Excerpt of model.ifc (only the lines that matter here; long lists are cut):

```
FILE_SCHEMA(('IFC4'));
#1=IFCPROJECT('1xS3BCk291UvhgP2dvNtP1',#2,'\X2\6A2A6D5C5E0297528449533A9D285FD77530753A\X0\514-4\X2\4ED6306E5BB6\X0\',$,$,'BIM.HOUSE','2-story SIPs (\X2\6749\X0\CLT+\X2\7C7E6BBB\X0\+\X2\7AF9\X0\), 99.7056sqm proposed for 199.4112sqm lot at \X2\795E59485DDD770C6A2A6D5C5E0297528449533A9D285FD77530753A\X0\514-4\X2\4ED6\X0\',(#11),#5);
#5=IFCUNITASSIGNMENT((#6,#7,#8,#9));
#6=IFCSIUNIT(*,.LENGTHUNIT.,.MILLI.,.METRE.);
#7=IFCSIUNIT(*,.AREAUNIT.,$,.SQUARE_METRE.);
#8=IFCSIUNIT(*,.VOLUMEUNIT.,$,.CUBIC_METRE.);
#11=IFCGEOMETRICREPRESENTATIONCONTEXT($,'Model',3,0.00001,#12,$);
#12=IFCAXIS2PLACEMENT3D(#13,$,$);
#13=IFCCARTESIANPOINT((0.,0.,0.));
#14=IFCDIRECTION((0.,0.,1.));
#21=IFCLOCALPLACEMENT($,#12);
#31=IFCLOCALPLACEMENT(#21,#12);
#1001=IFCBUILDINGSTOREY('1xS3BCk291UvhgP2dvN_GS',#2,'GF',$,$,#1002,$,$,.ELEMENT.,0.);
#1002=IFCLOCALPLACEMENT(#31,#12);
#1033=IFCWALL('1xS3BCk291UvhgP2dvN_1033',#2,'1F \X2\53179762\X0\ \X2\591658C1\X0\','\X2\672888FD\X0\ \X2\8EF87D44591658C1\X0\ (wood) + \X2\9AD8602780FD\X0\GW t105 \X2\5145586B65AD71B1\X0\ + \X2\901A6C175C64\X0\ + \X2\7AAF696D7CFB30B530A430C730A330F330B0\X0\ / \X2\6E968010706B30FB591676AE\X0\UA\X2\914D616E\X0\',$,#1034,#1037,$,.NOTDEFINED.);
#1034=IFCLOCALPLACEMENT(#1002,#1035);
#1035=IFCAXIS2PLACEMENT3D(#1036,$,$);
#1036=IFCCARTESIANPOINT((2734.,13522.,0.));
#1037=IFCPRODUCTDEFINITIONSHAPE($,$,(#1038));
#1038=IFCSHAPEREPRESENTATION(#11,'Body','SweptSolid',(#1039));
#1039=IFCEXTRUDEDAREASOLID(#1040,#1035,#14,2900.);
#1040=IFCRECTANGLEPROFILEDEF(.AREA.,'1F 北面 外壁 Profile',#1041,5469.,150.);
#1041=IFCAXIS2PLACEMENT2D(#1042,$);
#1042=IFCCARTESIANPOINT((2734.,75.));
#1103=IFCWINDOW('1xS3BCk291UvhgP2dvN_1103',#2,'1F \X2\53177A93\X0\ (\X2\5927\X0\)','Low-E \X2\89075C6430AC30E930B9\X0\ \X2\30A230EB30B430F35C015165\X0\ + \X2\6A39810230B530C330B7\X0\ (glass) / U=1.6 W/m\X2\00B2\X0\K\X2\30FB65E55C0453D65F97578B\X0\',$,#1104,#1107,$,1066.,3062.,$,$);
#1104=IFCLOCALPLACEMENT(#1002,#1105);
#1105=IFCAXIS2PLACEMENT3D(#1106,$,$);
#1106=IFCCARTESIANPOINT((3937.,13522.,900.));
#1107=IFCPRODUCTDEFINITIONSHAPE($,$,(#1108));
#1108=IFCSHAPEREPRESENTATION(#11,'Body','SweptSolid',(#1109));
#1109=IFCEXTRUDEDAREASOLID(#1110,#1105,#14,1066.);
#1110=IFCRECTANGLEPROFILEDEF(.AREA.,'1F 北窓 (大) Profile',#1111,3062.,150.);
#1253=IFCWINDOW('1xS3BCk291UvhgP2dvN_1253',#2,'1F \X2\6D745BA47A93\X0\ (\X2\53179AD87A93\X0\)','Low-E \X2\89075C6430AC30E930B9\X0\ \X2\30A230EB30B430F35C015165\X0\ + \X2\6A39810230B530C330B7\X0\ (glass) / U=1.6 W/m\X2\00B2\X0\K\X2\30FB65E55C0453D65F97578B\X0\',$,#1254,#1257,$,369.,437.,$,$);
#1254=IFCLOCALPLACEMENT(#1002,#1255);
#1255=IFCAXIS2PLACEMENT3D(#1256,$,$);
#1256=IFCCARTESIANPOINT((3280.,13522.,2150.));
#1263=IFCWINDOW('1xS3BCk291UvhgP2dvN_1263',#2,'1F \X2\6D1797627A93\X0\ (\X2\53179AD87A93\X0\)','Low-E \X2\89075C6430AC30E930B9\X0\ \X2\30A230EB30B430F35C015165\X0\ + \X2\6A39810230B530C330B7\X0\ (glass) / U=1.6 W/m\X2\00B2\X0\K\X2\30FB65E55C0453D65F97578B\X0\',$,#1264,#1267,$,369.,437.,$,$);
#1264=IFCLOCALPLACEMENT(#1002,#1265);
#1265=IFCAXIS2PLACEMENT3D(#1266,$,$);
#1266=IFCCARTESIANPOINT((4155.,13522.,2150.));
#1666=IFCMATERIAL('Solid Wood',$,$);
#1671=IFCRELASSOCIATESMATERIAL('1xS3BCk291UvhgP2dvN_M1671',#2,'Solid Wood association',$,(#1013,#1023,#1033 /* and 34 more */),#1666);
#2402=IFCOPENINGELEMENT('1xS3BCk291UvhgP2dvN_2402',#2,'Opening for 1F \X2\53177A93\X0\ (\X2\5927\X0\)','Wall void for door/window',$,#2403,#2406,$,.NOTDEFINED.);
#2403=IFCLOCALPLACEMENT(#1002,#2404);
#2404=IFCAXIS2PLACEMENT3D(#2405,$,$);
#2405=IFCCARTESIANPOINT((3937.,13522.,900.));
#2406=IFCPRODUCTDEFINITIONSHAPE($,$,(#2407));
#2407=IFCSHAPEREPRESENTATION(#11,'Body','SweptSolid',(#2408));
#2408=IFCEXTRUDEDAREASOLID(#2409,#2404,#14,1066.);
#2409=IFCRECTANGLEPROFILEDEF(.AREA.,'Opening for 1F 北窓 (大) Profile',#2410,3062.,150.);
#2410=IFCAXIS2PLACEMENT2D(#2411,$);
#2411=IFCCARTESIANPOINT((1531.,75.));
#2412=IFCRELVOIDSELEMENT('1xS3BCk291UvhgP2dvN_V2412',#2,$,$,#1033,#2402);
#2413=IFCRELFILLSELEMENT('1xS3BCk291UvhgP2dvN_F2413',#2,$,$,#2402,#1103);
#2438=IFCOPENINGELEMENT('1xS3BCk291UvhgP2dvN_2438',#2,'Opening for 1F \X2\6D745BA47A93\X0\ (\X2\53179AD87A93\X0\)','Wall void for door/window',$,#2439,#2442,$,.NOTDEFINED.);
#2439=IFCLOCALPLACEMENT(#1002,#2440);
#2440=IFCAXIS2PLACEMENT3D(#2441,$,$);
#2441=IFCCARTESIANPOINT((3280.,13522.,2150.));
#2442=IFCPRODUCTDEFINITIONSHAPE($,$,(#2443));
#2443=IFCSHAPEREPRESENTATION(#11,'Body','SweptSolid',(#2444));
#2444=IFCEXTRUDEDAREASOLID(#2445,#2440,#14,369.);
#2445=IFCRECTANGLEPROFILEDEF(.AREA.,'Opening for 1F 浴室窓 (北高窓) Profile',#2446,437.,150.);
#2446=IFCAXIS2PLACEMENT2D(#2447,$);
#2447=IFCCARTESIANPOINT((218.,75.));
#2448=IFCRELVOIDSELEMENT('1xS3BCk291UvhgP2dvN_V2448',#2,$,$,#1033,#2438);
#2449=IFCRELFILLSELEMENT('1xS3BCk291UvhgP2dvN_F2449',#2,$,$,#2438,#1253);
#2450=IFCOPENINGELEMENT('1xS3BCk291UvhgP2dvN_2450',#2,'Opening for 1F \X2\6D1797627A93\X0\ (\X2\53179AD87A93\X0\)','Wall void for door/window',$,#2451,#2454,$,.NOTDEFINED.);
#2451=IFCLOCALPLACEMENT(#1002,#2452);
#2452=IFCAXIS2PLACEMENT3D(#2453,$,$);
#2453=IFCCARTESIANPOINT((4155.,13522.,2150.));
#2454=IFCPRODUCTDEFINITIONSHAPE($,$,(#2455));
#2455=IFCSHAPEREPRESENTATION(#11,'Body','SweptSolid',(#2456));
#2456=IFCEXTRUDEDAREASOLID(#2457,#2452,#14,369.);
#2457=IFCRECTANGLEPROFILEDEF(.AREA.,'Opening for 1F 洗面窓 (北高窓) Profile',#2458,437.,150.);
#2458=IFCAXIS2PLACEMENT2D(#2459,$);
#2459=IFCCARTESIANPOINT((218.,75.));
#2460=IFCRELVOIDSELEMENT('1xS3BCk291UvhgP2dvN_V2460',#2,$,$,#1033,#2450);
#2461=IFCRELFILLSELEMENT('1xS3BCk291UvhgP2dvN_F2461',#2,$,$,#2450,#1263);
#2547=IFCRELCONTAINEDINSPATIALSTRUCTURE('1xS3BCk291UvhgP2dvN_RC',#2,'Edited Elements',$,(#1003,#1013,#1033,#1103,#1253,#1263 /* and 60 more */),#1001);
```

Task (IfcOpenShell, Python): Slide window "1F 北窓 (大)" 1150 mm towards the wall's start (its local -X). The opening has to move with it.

```python
import ifcopenshell
import ifcopenshell.api.geometry
import ifcopenshell.util.placement
import ifcopenshell.util.unit

model = ifcopenshell.open("model.ifc")
unit_scale = ifcopenshell.util.unit.calculate_unit_scale(model)

window = model.by_guid("1xS3BCk291UvhgP2dvN_1103")
opening = window.FillsVoids[0].RelatingOpeningElement
wall = opening.VoidsElements[0].RelatingBuildingElement

wall_matrix = ifcopenshell.util.placement.get_local_placement(wall.ObjectPlacement)
shift = wall_matrix[:3, 0] * -1.15 / unit_scale
before = ifcopenshell.util.placement.get_local_placement(window.ObjectPlacement)[:3, 3].copy()

# The window is not placed relative to its opening, so move both.
for product in (opening, window):
    matrix = ifcopenshell.util.placement.get_local_placement(product.ObjectPlacement)
    matrix[:3, 3] += shift
    ifcopenshell.api.geometry.edit_object_placement(model, product=product, matrix=matrix, is_si=False)

after = ifcopenshell.util.placement.get_local_placement(window.ObjectPlacement)[:3, 3]
print("window moved by", (after - before).round(3) + 0.0)

model.write("model_v2.ifc")
```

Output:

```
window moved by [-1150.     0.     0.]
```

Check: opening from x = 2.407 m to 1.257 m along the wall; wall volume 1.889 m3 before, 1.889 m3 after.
